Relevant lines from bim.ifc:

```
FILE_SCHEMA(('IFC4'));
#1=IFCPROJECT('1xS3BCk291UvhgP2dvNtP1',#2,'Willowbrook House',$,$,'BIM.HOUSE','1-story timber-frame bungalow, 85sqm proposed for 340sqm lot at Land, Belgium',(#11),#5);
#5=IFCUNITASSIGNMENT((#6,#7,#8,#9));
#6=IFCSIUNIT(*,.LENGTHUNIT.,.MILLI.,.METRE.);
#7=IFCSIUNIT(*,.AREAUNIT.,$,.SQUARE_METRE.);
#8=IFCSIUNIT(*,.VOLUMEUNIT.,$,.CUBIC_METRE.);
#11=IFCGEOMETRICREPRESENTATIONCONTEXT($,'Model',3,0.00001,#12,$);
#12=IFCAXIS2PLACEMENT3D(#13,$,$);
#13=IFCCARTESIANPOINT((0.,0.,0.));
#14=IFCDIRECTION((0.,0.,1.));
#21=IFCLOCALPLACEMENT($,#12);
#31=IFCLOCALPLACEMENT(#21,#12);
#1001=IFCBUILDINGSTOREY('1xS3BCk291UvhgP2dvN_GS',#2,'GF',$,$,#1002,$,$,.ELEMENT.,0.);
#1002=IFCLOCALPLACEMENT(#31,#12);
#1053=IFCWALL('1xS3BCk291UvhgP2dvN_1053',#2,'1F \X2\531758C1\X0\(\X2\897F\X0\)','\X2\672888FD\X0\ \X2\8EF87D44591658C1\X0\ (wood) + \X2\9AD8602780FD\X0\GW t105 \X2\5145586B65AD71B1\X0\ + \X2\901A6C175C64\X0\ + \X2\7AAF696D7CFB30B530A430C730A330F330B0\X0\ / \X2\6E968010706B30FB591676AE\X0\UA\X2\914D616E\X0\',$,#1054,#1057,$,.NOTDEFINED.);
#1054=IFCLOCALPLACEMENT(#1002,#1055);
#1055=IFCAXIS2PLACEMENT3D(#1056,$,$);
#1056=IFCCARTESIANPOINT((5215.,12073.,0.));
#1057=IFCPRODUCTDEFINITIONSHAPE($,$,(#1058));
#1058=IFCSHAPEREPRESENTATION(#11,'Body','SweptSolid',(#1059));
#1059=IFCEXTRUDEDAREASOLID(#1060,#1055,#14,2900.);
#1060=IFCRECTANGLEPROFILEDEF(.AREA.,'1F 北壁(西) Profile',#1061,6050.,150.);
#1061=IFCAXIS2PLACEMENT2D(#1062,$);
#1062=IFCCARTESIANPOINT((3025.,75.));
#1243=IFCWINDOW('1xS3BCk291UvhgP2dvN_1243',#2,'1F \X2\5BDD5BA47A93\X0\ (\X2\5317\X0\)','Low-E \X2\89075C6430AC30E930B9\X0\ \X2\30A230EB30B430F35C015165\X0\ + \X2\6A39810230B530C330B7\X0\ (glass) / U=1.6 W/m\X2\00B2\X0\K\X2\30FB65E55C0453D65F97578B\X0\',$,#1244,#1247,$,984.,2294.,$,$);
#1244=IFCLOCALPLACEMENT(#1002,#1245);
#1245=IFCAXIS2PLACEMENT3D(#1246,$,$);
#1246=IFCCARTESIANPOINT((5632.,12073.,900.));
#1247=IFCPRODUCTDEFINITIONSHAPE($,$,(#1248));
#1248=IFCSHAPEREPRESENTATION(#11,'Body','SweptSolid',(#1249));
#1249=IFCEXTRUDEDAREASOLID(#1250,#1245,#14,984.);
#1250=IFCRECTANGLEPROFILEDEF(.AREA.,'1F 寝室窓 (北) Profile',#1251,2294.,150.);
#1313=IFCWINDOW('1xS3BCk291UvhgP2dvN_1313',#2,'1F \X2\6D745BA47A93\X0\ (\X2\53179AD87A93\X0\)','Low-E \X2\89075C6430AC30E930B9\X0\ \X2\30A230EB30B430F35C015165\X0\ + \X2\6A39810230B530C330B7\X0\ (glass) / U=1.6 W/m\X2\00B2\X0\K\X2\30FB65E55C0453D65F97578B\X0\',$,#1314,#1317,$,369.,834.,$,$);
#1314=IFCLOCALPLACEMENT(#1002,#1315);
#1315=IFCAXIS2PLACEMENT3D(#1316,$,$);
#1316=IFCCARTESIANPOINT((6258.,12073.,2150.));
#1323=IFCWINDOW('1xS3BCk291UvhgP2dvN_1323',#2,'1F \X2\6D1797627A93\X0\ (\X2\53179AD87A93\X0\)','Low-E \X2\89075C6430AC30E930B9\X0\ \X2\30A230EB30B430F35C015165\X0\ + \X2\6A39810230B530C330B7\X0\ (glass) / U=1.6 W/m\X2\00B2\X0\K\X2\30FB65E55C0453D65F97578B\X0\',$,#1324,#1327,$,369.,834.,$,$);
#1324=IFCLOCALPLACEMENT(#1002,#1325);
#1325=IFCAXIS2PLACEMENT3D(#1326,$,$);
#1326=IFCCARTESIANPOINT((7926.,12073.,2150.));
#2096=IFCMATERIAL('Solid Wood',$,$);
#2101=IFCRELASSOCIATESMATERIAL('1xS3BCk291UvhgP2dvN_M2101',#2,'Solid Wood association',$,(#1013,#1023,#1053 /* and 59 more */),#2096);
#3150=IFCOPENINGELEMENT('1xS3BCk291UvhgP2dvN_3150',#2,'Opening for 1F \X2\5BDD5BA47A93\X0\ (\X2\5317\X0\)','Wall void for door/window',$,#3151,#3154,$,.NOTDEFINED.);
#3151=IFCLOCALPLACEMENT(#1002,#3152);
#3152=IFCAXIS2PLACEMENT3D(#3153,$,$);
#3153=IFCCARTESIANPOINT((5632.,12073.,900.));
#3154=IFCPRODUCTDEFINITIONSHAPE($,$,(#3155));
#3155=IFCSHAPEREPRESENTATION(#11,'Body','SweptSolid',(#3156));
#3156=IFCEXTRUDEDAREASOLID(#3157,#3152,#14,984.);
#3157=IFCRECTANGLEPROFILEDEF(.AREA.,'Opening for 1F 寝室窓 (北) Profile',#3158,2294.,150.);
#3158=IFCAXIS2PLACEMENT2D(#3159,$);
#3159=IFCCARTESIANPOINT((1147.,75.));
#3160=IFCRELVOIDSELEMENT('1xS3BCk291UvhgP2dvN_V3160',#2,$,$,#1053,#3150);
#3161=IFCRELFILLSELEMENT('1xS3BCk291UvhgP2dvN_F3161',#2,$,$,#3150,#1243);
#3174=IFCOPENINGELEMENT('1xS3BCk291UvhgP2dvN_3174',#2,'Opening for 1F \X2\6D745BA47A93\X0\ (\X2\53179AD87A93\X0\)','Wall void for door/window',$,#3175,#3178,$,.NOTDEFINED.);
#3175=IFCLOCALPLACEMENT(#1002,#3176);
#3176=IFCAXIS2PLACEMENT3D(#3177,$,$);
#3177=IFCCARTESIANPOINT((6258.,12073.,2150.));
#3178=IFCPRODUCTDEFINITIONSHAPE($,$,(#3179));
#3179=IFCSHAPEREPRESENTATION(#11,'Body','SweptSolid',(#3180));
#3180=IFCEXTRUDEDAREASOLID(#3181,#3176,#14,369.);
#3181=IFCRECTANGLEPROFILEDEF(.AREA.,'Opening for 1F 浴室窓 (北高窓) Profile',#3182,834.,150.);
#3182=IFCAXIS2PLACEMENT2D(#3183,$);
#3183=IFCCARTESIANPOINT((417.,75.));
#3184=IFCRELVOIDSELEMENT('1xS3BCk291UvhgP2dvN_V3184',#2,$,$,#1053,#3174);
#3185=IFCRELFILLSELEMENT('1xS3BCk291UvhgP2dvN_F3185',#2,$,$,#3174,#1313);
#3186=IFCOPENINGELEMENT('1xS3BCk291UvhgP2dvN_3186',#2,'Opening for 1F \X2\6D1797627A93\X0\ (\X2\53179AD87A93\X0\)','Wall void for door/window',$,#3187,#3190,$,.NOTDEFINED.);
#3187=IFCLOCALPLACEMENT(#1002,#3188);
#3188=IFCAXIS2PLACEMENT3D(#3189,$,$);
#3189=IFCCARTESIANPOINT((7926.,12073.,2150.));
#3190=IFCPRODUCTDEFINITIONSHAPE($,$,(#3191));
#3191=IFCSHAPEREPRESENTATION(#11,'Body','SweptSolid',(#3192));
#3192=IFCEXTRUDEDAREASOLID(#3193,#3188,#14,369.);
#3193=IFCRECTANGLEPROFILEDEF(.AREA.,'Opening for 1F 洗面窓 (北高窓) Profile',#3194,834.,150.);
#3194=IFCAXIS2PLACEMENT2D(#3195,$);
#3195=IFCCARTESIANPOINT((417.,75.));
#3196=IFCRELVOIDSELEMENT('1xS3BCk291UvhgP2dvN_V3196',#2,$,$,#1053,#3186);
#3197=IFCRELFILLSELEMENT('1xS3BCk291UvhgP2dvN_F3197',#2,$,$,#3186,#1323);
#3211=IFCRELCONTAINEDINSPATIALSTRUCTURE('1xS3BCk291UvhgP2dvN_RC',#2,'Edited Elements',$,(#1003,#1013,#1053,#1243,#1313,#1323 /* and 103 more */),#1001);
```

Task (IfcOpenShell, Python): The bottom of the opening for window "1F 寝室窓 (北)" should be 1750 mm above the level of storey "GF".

```python
import numpy as np
import ifcopenshell
import ifcopenshell.api.geometry
import ifcopenshell.geom
import ifcopenshell.util.element
import ifcopenshell.util.placement
import ifcopenshell.util.shape
import ifcopenshell.util.unit

model = ifcopenshell.open("bim.ifc")
unit_scale = ifcopenshell.util.unit.calculate_unit_scale(model)

window = model.by_guid("1xS3BCk291UvhgP2dvN_1243")
opening = window.FillsVoids[0].RelatingOpeningElement
storey = ifcopenshell.util.element.get_container(window, ifc_class="IfcBuildingStorey")
level = ifcopenshell.util.placement.get_local_placement(storey.ObjectPlacement)[2, 3]

# The opening's origin need not be at the sill, so measure its lowest point.
shape = ifcopenshell.geom.create_shape(ifcopenshell.geom.settings(), opening)
bottom = ifcopenshell.util.shape.get_shape_bottom_elevation(shape, shape.geometry) / unit_scale
dz = level + 1750.0 - bottom

shift = np.array([0.0, 0.0, dz])
# The window is not placed relative to its opening, so move both.
for product in (opening, window):
    matrix = ifcopenshell.util.placement.get_local_placement(product.ObjectPlacement)
    matrix[:3, 3] += shift
    ifcopenshell.api.geometry.edit_object_placement(model, product=product, matrix=matrix, is_si=False)

print(f"moved by {dz * unit_scale:+.3f} m")

model.write("bim_updated.ifc")
```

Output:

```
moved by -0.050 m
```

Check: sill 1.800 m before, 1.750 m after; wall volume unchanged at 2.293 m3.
